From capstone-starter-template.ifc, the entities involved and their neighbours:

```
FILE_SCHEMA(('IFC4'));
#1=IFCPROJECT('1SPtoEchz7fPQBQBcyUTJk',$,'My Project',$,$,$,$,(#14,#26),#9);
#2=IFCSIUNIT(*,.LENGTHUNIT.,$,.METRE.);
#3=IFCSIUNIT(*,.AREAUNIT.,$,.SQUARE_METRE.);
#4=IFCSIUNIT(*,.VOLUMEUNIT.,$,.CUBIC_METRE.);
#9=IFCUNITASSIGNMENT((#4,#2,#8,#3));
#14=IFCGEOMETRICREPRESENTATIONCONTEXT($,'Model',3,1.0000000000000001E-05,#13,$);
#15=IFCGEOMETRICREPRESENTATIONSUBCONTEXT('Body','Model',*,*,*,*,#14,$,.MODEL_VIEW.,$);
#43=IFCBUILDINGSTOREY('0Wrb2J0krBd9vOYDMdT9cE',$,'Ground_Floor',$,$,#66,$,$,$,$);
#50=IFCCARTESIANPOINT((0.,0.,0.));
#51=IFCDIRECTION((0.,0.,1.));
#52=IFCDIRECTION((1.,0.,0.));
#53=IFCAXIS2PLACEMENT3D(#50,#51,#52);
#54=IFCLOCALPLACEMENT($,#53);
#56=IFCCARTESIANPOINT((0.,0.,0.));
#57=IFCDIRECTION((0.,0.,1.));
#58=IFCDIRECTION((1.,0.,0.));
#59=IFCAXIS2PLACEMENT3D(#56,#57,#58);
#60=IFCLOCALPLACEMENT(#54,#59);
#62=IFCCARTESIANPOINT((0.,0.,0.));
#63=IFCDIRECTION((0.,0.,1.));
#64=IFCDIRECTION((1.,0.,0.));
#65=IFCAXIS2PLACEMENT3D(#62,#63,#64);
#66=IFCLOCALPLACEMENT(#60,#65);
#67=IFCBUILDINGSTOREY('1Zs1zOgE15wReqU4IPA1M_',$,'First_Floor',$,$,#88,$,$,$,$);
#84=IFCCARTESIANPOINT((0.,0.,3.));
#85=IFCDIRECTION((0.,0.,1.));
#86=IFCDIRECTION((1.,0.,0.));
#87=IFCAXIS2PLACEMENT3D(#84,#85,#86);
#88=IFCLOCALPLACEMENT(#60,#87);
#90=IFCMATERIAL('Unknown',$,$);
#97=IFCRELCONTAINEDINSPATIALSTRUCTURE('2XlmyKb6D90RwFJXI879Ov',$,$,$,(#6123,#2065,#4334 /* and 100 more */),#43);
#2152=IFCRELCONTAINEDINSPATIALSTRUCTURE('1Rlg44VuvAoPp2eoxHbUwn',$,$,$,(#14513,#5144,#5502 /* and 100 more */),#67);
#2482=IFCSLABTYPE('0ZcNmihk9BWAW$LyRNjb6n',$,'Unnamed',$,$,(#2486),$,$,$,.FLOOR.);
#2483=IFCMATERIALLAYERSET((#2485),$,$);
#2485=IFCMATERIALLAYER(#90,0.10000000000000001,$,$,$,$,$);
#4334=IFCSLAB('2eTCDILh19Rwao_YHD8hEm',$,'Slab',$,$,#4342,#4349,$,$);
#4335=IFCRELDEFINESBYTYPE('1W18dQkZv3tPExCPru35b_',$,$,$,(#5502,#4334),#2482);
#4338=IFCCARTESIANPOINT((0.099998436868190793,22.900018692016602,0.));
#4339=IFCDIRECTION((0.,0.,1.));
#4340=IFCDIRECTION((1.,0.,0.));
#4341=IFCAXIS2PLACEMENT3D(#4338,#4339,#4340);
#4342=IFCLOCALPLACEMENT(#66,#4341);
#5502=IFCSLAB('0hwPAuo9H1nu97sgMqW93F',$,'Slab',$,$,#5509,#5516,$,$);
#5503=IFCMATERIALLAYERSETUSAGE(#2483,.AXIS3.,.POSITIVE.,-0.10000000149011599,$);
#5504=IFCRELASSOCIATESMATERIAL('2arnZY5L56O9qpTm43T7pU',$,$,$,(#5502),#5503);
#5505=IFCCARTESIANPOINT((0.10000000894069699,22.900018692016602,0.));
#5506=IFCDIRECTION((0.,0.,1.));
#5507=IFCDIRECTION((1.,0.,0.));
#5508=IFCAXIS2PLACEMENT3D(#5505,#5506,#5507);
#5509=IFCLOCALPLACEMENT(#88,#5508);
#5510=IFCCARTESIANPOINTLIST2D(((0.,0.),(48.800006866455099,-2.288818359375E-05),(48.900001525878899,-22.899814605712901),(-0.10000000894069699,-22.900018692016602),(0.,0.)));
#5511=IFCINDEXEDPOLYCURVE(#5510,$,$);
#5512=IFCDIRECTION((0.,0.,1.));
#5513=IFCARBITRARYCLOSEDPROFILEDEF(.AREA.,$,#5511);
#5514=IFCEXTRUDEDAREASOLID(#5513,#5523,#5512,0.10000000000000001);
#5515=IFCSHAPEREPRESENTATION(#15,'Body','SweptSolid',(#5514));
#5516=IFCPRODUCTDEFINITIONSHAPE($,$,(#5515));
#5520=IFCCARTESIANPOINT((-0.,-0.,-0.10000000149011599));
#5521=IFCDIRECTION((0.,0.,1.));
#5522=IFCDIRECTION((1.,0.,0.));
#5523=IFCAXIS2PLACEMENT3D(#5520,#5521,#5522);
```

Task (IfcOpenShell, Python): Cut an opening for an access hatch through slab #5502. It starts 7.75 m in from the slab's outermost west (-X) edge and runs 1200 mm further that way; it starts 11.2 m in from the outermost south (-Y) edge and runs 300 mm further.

```python
import numpy as np
import ifcopenshell
import ifcopenshell.api.feature
import ifcopenshell.api.geometry
import ifcopenshell.api.root
import ifcopenshell.geom
import ifcopenshell.util.placement
import ifcopenshell.util.representation
import ifcopenshell.util.shape
import ifcopenshell.util.unit

model = ifcopenshell.open("capstone-starter-template.ifc")
unit_scale = ifcopenshell.util.unit.calculate_unit_scale(model)
settings = ifcopenshell.geom.settings()


def volume(element):
    """Net volume in cubic metres, openings subtracted."""
    shape = ifcopenshell.geom.create_shape(settings, element)
    return ifcopenshell.util.shape.get_volume(shape.geometry)


slab = model.by_guid("0hwPAuo9H1nu97sgMqW93F")
before = volume(slab)

# Extent in the slab's own axes, in metres. The edges named are its -X and -Y sides.
slab_shape = ifcopenshell.geom.create_shape(settings, slab)
vertices = ifcopenshell.util.shape.get_vertices(slab_shape.geometry)
x_min, y_min, bottom = vertices.min(axis=0)
top = vertices[:, 2].max()

opening = ifcopenshell.api.root.create_entity(model, ifc_class="IfcOpeningElement", name="Access hatch opening", predefined_type="OPENING")
context = ifcopenshell.util.representation.get_context(model, "Model", "Body", "MODEL_VIEW")
width, depth = 1.2, 0.3
outline = [(0.0, 0.0), (width, 0.0), (width, depth), (0.0, depth), (0.0, 0.0)]
# Overshoot both faces by 50 mm so the cut is clean.
shape = ifcopenshell.api.geometry.add_slab_representation(
    model, context=context, depth=top - bottom + 0.1, polyline=outline
)
ifcopenshell.api.geometry.assign_representation(model, product=opening, representation=shape)

matrix = ifcopenshell.util.placement.get_local_placement(slab.ObjectPlacement)
matrix[:, 3] = matrix @ np.append(np.array([x_min + 7.75, y_min + 11.2, bottom - 0.05]) / unit_scale, 1.0)
ifcopenshell.api.geometry.edit_object_placement(model, product=opening, matrix=matrix, is_si=False)
ifcopenshell.api.feature.add_feature(model, feature=opening, element=slab)

after = volume(slab)

print(f"slab volume {before:.3f} -> {after:.3f} m3")

model.write("capstone-starter-template-out.ifc")
```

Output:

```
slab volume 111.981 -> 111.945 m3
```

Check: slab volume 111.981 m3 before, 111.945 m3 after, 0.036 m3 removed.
